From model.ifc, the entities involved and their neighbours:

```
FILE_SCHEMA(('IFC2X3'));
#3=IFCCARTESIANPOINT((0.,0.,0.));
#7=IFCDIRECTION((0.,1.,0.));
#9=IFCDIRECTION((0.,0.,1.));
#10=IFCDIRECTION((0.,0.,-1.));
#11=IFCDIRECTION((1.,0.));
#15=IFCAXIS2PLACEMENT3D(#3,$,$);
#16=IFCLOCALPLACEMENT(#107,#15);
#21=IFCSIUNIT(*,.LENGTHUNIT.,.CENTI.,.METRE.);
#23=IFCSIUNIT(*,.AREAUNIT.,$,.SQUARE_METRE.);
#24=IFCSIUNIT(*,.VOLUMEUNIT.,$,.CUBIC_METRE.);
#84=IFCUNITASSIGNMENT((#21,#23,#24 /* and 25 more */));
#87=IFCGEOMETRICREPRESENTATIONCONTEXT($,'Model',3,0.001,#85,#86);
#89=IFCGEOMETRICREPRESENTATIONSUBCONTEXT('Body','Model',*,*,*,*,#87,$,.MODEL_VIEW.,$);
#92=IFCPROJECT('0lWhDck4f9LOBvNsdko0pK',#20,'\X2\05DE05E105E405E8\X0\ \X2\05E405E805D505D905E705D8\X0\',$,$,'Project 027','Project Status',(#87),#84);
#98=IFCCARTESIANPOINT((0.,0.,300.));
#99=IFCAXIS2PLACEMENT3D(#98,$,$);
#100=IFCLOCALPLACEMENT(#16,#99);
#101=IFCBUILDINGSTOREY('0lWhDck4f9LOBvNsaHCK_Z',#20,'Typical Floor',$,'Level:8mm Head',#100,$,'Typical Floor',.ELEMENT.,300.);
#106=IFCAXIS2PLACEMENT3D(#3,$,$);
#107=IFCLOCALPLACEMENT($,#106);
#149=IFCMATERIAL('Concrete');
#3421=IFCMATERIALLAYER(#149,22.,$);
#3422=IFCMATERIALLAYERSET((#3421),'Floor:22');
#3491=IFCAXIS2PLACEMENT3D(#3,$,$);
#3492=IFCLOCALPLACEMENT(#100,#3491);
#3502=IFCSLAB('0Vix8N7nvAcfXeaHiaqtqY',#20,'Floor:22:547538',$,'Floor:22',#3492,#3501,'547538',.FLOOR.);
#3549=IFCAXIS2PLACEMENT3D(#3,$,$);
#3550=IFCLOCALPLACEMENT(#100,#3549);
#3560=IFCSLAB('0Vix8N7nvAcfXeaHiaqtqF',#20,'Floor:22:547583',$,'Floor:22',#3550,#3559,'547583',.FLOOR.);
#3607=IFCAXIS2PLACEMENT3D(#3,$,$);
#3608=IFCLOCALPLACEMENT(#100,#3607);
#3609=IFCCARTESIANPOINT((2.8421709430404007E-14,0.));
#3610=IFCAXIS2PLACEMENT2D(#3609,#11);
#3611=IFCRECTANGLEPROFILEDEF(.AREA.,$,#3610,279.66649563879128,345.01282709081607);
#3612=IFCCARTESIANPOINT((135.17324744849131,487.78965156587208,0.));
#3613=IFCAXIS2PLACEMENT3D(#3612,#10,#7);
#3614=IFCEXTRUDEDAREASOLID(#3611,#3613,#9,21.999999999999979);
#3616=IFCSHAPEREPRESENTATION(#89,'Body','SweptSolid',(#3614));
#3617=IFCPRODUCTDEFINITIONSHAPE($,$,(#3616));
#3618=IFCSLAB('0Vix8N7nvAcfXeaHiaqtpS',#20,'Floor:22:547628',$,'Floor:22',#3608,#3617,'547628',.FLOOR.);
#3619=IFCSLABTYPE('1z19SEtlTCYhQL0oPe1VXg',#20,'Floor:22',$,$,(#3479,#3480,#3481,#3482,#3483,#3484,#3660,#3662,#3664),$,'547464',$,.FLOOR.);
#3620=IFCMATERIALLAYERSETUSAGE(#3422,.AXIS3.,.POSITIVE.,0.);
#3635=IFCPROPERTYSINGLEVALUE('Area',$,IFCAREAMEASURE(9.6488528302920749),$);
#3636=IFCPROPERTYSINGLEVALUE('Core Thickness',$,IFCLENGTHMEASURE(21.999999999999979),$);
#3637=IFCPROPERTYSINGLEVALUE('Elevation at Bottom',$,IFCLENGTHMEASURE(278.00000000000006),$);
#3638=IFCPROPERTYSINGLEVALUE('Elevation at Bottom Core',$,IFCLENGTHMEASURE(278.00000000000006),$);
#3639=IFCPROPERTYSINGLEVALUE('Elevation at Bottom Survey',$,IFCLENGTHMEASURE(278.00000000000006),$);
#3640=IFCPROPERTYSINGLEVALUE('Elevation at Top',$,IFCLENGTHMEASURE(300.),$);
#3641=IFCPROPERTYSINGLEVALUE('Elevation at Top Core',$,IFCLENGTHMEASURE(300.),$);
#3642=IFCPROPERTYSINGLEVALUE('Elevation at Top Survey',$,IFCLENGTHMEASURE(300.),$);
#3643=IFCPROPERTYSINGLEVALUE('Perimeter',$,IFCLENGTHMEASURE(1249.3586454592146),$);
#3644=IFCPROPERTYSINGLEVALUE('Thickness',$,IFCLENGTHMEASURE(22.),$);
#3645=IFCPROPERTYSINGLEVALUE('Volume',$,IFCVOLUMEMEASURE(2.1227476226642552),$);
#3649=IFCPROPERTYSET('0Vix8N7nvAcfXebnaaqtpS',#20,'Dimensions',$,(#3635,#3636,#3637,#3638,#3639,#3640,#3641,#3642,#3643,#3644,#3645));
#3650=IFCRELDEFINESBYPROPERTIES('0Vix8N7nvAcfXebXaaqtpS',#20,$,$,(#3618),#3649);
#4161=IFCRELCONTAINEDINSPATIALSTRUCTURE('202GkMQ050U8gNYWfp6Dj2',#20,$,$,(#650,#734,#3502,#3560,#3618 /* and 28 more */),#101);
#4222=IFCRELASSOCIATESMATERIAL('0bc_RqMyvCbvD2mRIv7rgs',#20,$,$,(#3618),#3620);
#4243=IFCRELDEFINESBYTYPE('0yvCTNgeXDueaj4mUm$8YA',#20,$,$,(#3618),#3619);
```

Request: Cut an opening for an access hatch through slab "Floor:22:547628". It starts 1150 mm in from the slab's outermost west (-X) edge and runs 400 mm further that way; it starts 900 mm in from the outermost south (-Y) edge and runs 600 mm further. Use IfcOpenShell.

```python
import numpy as np
import ifcopenshell
import ifcopenshell.api.feature
import ifcopenshell.api.geometry
import ifcopenshell.api.pset
import ifcopenshell.api.root
import ifcopenshell.geom
import ifcopenshell.util.element
import ifcopenshell.util.placement
import ifcopenshell.util.representation
import ifcopenshell.util.shape
import ifcopenshell.util.unit

model = ifcopenshell.open("model.ifc")
unit_scale = ifcopenshell.util.unit.calculate_unit_scale(model)
area_scale = ifcopenshell.util.unit.calculate_unit_scale(model, "AREAUNIT")
volume_scale = ifcopenshell.util.unit.calculate_unit_scale(model, "VOLUMEUNIT")
settings = ifcopenshell.geom.settings()


def volume(element):
    """Net volume in cubic metres, openings subtracted."""
    shape = ifcopenshell.geom.create_shape(settings, element)
    return ifcopenshell.util.shape.get_volume(shape.geometry)


slab = model.by_guid("0Vix8N7nvAcfXeaHiaqtpS")
before = volume(slab)

# Extent in the slab's own axes, in metres. The edges named are its -X and -Y sides.
slab_shape = ifcopenshell.geom.create_shape(settings, slab)
vertices = ifcopenshell.util.shape.get_vertices(slab_shape.geometry)
x_min, y_min, bottom = vertices.min(axis=0)
top = vertices[:, 2].max()

opening = ifcopenshell.api.root.create_entity(model, ifc_class="IfcOpeningElement", name="Access hatch opening")
context = ifcopenshell.util.representation.get_context(model, "Model", "Body", "MODEL_VIEW")
width, depth = 0.4, 0.6
outline = [(0.0, 0.0), (width, 0.0), (width, depth), (0.0, depth), (0.0, 0.0)]
# Overshoot both faces by 50 mm so the cut is clean.
shape = ifcopenshell.api.geometry.add_slab_representation(
    model, context=context, depth=top - bottom + 0.1, polyline=outline
)
ifcopenshell.api.geometry.assign_representation(model, product=opening, representation=shape)

matrix = ifcopenshell.util.placement.get_local_placement(slab.ObjectPlacement)
matrix[:, 3] = matrix @ np.append(np.array([x_min + 1.15, y_min + 0.9, bottom - 0.05]) / unit_scale, 1.0)
ifcopenshell.api.geometry.edit_object_placement(model, product=opening, matrix=matrix, is_si=False)
ifcopenshell.api.feature.add_feature(model, feature=opening, element=slab)

after = volume(slab)

# Update the slab's stored quantities.
pset = model.by_id(ifcopenshell.util.element.get_pset(slab, "Dimensions", should_inherit=False)["id"])
ifcopenshell.api.pset.edit_pset(model, pset=pset, properties={
    "Area": model.create_entity("IfcAreaMeasure", after / (top - bottom) / area_scale),
    "Volume": model.create_entity("IfcVolumeMeasure", after / volume_scale),
})

print(f"slab volume {before:.3f} -> {after:.3f} m3")

model.write("model_updated.ifc")
```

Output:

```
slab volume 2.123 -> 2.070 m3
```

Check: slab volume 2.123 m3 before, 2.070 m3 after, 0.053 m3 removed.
